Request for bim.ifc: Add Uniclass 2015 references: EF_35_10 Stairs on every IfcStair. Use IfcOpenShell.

First a look at what the model holds.

```python
import ifcopenshell

model = ifcopenshell.open("bim.ifc")
print(model.schema)
print("classifications:", [c.Name for c in model.by_type("IfcClassification")])
for ifc_class in ("IfcDoor", "IfcRoof", "IfcStair", "IfcWall", "IfcWindow"):
    print(ifc_class, len(model.by_type(ifc_class)))
```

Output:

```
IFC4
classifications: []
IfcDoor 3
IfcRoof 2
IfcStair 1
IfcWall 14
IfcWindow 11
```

```python
import ifcopenshell
import ifcopenshell.api.classification

model = ifcopenshell.open("bim.ifc")

system = ifcopenshell.api.classification.add_classification(model, classification="Uniclass 2015")

codes = {
    "IfcStair": ("EF_35_10", "Stairs"),
}
for ifc_class, (code, name) in codes.items():
    products = model.by_type(ifc_class)
    ifcopenshell.api.classification.add_reference(
        model, products=products, classification=system, identification=code, name=name
    )
    print(code, len(products))

model.write("bim_edited.ifc")
```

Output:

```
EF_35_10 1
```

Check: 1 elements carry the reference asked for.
